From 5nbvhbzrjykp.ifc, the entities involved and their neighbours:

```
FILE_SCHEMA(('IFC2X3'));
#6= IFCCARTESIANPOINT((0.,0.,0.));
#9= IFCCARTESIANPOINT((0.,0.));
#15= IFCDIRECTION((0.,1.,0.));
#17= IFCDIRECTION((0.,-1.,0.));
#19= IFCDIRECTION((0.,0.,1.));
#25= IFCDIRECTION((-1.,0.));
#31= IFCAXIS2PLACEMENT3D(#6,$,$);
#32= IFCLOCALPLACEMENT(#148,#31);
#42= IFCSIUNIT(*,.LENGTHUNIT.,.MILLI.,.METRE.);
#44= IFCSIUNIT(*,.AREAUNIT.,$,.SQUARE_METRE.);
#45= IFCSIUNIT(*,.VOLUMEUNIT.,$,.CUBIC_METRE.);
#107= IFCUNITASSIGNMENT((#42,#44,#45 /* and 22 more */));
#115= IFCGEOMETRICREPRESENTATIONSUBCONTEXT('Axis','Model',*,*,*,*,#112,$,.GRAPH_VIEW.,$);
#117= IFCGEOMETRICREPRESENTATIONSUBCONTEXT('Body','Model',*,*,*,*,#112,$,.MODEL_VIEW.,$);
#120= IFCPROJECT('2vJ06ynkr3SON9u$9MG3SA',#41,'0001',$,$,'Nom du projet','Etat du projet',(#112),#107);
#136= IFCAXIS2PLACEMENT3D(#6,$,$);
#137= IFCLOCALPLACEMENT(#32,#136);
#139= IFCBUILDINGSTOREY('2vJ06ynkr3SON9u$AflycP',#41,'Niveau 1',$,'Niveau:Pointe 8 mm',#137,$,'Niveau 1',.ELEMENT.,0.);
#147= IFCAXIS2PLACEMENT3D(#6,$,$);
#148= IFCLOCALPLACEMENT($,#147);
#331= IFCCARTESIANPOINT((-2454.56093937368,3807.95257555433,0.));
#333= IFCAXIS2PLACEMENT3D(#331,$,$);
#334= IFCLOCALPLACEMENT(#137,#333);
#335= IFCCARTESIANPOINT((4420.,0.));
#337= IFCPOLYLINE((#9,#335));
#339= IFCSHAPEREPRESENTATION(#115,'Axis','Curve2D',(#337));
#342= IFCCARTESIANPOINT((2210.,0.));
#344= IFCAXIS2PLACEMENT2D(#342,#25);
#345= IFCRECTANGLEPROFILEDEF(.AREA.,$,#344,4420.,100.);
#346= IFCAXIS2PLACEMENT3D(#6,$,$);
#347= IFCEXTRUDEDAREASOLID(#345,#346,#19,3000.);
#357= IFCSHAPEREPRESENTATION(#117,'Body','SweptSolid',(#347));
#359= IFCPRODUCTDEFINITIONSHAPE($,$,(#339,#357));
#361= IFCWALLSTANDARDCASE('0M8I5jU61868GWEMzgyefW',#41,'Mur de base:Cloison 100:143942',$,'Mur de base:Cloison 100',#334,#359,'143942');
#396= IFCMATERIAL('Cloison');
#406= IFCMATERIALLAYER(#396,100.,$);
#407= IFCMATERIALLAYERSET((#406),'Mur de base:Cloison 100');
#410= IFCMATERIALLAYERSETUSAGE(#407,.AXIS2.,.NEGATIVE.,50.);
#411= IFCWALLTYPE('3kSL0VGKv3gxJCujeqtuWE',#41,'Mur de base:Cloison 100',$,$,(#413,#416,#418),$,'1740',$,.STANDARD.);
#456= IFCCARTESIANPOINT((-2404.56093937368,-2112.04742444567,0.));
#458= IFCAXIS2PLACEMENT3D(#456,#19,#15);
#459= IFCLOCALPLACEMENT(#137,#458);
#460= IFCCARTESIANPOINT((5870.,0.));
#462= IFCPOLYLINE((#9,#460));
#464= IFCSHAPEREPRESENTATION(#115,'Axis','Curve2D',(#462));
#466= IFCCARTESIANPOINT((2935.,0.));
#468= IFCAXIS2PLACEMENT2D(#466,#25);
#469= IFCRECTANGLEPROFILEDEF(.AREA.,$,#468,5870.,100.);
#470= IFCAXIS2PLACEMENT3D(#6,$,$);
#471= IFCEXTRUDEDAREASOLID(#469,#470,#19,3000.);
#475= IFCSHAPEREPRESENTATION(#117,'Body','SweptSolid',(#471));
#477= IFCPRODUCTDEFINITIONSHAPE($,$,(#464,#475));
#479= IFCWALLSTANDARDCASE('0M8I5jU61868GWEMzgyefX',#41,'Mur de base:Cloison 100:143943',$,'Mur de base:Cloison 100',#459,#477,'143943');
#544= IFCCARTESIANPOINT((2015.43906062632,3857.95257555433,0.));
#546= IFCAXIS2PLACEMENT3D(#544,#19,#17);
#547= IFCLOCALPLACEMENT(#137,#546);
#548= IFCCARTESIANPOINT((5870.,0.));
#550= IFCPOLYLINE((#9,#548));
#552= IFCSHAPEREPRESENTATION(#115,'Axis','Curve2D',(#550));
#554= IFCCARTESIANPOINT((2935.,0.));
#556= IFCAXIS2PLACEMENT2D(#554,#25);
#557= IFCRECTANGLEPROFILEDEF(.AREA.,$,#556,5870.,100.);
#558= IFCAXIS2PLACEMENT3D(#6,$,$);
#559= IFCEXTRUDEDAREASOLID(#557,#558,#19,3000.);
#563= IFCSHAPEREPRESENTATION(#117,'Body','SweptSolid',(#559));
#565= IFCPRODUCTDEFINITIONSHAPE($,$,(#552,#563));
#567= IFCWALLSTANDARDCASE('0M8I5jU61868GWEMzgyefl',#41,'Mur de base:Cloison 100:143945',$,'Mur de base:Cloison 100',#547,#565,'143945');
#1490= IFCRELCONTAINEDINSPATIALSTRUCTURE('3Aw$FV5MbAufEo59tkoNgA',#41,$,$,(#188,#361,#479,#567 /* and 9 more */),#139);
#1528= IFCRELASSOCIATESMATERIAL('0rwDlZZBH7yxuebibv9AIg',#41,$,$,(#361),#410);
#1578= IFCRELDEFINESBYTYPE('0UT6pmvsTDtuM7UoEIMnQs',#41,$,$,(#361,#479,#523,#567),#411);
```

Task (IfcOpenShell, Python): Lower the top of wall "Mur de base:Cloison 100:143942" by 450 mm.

```python
import ifcopenshell
import ifcopenshell.geom
import ifcopenshell.util.representation
import ifcopenshell.util.shape
import ifcopenshell.util.unit

model = ifcopenshell.open("5nbvhbzrjykp.ifc")
unit_scale = ifcopenshell.util.unit.calculate_unit_scale(model)
settings = ifcopenshell.geom.settings()


def volume(element):
    """Net volume in cubic metres, openings subtracted."""
    shape = ifcopenshell.geom.create_shape(settings, element)
    return ifcopenshell.util.shape.get_volume(shape.geometry)


wall = model.by_id(361)
before = volume(wall)

body = ifcopenshell.util.representation.get_representation(wall, "Model", "Body")
solid = body.Items[0]
old_height = solid.Depth
solid.Depth -= 0.45 / unit_scale
after = volume(wall)

print(f"height {old_height:g} -> {solid.Depth:g}, volume {before:.3f} -> {after:.3f} m3")

model.write("5nbvhbzrjykp_rev.ifc")
```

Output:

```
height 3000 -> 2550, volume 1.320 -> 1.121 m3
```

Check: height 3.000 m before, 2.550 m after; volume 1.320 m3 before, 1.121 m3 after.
